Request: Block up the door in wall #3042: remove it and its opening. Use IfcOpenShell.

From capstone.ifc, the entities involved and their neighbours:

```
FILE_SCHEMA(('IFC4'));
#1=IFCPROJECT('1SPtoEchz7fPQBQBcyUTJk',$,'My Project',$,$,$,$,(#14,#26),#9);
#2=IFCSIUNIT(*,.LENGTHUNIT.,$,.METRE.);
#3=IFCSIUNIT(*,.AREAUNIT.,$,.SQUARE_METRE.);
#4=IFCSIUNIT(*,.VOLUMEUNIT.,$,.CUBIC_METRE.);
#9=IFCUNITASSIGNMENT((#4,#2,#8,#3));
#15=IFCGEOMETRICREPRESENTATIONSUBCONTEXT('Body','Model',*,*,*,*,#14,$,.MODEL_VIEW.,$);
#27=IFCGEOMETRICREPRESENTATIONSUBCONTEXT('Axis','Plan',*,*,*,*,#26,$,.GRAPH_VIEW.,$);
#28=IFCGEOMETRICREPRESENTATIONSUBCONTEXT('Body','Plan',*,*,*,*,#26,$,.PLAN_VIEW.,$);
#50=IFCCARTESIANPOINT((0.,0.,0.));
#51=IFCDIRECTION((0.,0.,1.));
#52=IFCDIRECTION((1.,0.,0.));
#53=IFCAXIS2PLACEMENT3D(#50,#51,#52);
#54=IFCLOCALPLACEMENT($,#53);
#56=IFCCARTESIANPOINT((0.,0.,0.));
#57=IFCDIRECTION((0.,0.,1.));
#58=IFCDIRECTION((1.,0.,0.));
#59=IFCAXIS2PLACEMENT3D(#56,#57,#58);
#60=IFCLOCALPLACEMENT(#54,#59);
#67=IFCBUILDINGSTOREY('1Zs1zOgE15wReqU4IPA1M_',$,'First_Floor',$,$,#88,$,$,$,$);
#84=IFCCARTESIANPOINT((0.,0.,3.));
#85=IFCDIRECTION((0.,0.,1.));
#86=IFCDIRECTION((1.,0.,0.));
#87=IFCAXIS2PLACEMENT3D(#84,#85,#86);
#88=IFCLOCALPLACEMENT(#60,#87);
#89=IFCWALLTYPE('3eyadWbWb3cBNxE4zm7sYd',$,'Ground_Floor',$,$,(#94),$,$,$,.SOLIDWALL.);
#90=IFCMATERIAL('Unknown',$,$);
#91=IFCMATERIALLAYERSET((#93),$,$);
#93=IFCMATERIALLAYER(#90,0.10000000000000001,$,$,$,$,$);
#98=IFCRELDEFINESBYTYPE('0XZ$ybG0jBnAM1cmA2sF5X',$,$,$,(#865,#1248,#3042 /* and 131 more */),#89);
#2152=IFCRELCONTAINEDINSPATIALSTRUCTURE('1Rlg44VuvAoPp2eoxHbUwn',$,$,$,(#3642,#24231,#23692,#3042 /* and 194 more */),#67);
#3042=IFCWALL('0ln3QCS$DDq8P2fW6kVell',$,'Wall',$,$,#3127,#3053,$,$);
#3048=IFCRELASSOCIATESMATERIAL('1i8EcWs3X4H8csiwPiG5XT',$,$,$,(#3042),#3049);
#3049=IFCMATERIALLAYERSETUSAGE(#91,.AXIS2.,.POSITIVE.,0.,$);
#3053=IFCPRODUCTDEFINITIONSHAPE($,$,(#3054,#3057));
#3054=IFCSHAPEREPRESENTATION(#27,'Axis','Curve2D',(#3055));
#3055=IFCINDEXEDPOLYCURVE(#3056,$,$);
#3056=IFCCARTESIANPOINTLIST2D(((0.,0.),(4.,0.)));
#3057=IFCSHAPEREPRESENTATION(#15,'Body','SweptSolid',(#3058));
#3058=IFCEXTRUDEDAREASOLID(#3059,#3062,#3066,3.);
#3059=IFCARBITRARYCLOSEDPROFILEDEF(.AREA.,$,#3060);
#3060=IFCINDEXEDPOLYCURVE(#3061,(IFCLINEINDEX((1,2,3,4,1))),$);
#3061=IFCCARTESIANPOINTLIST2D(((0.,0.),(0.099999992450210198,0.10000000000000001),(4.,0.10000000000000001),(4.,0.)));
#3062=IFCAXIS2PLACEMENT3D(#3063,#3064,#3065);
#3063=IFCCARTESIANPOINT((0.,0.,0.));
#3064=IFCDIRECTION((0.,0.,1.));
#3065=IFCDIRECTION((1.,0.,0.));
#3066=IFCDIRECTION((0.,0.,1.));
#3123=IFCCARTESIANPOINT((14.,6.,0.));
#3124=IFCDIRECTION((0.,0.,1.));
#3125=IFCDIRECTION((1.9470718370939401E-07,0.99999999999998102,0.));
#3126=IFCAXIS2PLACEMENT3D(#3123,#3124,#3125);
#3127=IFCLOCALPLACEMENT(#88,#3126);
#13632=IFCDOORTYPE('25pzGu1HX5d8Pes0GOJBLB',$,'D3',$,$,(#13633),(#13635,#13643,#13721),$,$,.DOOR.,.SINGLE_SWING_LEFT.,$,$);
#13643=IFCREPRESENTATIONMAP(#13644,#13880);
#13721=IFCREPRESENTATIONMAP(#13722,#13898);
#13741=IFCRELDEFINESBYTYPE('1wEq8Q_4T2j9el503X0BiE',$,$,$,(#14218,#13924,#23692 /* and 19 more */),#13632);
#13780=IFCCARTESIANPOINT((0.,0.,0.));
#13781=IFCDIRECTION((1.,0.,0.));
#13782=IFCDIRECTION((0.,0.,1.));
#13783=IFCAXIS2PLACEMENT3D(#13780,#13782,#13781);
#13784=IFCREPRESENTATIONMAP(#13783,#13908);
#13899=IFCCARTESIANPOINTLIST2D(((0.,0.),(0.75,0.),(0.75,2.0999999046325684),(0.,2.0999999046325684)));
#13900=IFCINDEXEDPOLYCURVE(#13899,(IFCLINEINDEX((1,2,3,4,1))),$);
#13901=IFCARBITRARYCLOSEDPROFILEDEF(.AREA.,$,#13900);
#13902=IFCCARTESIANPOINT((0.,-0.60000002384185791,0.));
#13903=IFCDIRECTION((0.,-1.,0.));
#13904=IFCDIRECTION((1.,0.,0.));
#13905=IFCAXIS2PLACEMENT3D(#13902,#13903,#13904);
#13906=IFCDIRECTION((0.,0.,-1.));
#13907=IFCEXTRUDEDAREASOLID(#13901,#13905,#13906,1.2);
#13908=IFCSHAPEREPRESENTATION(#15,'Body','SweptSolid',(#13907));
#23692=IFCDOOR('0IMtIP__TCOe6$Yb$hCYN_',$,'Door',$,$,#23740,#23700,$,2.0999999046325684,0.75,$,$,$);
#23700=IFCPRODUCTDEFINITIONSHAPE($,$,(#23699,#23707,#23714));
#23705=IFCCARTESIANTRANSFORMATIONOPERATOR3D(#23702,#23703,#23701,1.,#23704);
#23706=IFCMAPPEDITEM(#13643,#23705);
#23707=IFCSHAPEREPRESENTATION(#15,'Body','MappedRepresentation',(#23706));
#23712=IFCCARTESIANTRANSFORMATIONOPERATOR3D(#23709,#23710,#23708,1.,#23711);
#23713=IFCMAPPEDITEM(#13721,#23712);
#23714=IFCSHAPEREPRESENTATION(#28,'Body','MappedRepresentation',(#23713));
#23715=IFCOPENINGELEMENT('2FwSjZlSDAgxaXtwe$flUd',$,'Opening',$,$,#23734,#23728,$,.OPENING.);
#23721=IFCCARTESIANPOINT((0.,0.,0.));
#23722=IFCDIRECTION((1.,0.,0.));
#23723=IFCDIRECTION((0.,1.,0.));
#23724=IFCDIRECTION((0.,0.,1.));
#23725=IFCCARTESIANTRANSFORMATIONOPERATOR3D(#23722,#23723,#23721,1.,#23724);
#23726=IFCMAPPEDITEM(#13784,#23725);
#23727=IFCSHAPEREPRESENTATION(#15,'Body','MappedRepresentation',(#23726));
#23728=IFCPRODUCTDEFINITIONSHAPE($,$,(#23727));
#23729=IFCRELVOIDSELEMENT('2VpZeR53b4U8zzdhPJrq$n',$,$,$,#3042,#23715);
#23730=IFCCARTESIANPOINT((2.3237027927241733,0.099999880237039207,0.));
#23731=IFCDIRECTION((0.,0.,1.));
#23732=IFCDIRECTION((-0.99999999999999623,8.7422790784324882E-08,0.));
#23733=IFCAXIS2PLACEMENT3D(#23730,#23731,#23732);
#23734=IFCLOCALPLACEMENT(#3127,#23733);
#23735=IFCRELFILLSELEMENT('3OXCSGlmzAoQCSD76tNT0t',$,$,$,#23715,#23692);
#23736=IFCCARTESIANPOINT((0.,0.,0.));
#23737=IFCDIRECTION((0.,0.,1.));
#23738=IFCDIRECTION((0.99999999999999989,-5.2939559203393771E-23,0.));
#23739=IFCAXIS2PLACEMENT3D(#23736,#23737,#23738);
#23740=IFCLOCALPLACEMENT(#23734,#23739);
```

```python
import ifcopenshell
import ifcopenshell.api.feature
import ifcopenshell.api.root
import ifcopenshell.geom
import ifcopenshell.util.shape

model = ifcopenshell.open("capstone.ifc")
settings = ifcopenshell.geom.settings()


def volume(element):
    """Net volume in cubic metres, openings subtracted."""
    shape = ifcopenshell.geom.create_shape(settings, element)
    return ifcopenshell.util.shape.get_volume(shape.geometry)


door = model.by_guid("0IMtIP__TCOe6$Yb$hCYN_")
opening = door.FillsVoids[0].RelatingOpeningElement
wall = opening.VoidsElements[0].RelatingBuildingElement
before = volume(wall)

ifcopenshell.api.root.remove_product(model, product=door)
ifcopenshell.api.feature.remove_feature(model, feature=opening)

after = volume(wall)

print(f"wall volume {before:.3f} -> {after:.3f} m3")

model.write("capstone-out.ifc")
```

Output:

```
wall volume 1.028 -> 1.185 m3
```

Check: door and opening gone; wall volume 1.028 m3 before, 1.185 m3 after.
